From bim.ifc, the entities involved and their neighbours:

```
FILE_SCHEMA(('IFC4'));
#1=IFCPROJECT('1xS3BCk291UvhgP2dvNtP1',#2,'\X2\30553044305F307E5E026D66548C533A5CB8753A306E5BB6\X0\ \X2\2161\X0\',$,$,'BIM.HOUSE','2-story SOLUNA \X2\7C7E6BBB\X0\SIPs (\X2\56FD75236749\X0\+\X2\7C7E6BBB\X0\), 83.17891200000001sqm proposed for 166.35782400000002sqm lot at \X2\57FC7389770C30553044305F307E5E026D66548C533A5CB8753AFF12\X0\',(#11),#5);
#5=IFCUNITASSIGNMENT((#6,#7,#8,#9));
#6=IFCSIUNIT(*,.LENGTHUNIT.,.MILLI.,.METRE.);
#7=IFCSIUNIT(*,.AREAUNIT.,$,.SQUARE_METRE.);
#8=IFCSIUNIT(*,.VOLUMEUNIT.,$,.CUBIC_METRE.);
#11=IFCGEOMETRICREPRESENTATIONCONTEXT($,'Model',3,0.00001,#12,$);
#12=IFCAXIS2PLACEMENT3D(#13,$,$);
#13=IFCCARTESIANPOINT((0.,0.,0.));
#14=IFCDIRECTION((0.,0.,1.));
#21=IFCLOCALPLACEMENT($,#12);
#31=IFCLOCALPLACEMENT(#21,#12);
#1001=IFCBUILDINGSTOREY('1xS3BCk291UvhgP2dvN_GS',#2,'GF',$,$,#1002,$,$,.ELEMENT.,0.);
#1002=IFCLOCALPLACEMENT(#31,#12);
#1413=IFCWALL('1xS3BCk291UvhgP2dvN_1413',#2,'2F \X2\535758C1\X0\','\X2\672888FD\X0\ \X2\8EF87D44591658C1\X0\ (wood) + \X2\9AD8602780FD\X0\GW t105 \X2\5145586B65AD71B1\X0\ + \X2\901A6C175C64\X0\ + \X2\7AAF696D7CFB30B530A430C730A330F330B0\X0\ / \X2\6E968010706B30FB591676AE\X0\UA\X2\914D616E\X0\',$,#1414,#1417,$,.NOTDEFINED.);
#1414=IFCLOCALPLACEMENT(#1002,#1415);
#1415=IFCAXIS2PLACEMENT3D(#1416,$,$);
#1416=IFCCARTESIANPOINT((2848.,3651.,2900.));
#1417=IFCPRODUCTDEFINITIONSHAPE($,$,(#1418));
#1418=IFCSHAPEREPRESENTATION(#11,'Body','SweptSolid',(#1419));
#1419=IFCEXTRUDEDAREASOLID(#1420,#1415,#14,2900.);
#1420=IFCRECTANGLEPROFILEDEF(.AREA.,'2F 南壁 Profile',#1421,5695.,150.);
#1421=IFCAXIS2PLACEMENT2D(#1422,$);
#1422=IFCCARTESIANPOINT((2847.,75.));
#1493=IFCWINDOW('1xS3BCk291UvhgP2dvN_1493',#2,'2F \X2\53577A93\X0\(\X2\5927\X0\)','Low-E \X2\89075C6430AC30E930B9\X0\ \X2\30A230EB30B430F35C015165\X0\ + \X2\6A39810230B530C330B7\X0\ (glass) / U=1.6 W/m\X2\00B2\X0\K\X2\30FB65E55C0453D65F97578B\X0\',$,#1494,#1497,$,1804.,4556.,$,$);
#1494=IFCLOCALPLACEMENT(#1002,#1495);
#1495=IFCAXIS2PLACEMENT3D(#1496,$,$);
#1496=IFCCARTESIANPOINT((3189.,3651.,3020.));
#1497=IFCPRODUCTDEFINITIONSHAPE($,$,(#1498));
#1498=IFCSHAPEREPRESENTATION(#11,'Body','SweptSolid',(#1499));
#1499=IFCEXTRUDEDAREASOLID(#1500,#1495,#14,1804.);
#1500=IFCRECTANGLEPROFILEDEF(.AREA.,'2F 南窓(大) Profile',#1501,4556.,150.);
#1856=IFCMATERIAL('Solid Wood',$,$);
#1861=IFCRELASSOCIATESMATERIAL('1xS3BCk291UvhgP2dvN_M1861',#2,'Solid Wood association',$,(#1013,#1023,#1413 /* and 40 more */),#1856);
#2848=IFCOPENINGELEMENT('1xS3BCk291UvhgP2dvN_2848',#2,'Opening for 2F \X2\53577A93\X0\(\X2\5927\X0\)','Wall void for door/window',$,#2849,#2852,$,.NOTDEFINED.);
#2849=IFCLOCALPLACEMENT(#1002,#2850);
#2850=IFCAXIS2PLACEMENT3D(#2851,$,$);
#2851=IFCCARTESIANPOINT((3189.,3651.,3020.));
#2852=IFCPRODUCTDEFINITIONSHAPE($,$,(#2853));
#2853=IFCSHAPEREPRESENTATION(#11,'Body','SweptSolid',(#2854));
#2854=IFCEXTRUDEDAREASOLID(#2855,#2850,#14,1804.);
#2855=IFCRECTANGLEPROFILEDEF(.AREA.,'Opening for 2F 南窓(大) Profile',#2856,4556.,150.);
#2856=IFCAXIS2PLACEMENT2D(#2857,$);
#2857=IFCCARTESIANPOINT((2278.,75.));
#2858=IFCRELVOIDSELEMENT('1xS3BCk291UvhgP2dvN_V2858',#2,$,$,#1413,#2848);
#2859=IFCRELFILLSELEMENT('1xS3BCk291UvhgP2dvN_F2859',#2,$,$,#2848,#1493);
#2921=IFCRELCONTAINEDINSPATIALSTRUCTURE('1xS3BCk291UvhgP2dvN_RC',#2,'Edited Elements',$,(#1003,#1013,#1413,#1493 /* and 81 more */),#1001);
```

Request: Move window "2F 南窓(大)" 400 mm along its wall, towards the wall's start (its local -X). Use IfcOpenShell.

```python
import ifcopenshell
import ifcopenshell.api.geometry
import ifcopenshell.util.placement
import ifcopenshell.util.unit

model = ifcopenshell.open("bim.ifc")
unit_scale = ifcopenshell.util.unit.calculate_unit_scale(model)

window = model.by_guid("1xS3BCk291UvhgP2dvN_1493")
opening = window.FillsVoids[0].RelatingOpeningElement
wall = opening.VoidsElements[0].RelatingBuildingElement

wall_matrix = ifcopenshell.util.placement.get_local_placement(wall.ObjectPlacement)
shift = wall_matrix[:3, 0] * -0.4 / unit_scale
before = ifcopenshell.util.placement.get_local_placement(window.ObjectPlacement)[:3, 3].copy()

# The window is not placed relative to its opening, so move both.
for product in (opening, window):
    matrix = ifcopenshell.util.placement.get_local_placement(product.ObjectPlacement)
    matrix[:3, 3] += shift
    ifcopenshell.api.geometry.edit_object_placement(model, product=product, matrix=matrix, is_si=False)

after = ifcopenshell.util.placement.get_local_placement(window.ObjectPlacement)[:3, 3]
print("window moved by", (after - before).round(3) + 0.0)

model.write("bim_updated.ifc")
```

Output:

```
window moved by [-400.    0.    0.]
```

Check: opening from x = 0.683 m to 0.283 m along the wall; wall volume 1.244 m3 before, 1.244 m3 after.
